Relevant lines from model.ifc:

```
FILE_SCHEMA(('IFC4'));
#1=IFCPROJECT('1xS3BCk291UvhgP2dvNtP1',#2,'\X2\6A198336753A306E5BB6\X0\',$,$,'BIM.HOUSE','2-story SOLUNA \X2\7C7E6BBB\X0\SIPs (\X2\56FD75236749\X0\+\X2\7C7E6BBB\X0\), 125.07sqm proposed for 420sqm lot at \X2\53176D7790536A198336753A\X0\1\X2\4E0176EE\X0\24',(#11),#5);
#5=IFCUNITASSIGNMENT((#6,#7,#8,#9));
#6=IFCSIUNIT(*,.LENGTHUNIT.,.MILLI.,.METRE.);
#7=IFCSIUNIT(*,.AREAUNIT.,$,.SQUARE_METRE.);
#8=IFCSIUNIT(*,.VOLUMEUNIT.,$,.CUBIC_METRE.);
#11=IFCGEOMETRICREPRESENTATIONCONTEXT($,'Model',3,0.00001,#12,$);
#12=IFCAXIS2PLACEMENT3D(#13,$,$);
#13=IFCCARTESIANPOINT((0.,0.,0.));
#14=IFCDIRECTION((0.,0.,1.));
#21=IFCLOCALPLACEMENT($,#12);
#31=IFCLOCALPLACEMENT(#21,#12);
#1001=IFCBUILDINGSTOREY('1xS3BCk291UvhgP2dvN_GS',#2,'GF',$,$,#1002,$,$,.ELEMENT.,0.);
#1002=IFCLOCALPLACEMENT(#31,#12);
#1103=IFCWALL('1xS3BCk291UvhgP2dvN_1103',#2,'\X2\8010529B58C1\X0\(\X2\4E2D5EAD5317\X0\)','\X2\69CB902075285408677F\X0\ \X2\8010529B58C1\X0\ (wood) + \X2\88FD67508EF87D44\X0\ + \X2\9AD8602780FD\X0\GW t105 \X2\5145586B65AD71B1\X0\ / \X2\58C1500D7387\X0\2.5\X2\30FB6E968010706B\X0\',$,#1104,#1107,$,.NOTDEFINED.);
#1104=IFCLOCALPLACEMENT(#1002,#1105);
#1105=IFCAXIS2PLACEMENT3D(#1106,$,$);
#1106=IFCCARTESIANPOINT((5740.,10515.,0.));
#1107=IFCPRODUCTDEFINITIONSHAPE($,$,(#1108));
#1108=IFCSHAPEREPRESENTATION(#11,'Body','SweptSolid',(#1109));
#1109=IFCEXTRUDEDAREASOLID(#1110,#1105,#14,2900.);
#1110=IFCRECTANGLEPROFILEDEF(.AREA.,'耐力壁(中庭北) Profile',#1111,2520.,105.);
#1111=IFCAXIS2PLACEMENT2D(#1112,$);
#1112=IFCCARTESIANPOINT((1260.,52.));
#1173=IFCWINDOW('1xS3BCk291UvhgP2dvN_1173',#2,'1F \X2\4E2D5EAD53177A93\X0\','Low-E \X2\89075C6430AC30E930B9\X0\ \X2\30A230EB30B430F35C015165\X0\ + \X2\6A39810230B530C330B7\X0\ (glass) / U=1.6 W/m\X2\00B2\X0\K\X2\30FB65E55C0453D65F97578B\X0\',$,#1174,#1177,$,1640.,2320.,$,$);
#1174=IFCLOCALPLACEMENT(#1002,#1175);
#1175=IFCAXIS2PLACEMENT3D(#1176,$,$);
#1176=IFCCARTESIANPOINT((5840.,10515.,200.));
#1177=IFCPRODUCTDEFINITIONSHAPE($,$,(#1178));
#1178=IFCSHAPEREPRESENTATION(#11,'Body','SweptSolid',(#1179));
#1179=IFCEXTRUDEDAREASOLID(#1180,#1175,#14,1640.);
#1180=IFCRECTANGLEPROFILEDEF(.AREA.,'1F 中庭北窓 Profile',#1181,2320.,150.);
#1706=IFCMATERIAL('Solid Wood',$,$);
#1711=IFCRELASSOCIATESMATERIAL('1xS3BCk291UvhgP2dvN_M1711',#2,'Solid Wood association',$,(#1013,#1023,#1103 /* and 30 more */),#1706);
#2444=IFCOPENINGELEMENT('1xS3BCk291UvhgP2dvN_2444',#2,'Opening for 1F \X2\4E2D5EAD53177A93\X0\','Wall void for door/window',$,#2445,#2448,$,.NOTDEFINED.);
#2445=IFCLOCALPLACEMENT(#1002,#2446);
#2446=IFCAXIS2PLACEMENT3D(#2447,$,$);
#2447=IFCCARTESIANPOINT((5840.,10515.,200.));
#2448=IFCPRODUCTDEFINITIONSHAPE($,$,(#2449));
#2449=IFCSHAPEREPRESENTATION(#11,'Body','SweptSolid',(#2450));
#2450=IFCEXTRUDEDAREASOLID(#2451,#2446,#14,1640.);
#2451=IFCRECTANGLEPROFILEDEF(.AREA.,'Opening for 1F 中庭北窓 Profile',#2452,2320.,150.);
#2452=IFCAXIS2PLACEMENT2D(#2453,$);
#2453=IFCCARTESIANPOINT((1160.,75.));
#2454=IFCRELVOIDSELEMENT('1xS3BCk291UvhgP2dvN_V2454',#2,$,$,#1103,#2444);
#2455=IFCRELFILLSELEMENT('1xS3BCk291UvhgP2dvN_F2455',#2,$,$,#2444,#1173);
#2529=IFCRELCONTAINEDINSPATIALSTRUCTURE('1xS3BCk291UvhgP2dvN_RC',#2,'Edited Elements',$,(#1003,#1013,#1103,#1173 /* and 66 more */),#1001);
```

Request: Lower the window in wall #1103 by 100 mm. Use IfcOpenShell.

```python
import numpy as np
import ifcopenshell
import ifcopenshell.api.geometry
import ifcopenshell.util.placement
import ifcopenshell.util.unit

model = ifcopenshell.open("model.ifc")
unit_scale = ifcopenshell.util.unit.calculate_unit_scale(model)

window = model.by_guid("1xS3BCk291UvhgP2dvN_1173")
opening = window.FillsVoids[0].RelatingOpeningElement
dz = -0.1 / unit_scale

shift = np.array([0.0, 0.0, dz])
# The window is not placed relative to its opening, so move both.
for product in (opening, window):
    matrix = ifcopenshell.util.placement.get_local_placement(product.ObjectPlacement)
    matrix[:3, 3] += shift
    ifcopenshell.api.geometry.edit_object_placement(model, product=product, matrix=matrix, is_si=False)

print(f"moved by {dz * unit_scale:+.3f} m")

model.write("model_rev.ifc")
```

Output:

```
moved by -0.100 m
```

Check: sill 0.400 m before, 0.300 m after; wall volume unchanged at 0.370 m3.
